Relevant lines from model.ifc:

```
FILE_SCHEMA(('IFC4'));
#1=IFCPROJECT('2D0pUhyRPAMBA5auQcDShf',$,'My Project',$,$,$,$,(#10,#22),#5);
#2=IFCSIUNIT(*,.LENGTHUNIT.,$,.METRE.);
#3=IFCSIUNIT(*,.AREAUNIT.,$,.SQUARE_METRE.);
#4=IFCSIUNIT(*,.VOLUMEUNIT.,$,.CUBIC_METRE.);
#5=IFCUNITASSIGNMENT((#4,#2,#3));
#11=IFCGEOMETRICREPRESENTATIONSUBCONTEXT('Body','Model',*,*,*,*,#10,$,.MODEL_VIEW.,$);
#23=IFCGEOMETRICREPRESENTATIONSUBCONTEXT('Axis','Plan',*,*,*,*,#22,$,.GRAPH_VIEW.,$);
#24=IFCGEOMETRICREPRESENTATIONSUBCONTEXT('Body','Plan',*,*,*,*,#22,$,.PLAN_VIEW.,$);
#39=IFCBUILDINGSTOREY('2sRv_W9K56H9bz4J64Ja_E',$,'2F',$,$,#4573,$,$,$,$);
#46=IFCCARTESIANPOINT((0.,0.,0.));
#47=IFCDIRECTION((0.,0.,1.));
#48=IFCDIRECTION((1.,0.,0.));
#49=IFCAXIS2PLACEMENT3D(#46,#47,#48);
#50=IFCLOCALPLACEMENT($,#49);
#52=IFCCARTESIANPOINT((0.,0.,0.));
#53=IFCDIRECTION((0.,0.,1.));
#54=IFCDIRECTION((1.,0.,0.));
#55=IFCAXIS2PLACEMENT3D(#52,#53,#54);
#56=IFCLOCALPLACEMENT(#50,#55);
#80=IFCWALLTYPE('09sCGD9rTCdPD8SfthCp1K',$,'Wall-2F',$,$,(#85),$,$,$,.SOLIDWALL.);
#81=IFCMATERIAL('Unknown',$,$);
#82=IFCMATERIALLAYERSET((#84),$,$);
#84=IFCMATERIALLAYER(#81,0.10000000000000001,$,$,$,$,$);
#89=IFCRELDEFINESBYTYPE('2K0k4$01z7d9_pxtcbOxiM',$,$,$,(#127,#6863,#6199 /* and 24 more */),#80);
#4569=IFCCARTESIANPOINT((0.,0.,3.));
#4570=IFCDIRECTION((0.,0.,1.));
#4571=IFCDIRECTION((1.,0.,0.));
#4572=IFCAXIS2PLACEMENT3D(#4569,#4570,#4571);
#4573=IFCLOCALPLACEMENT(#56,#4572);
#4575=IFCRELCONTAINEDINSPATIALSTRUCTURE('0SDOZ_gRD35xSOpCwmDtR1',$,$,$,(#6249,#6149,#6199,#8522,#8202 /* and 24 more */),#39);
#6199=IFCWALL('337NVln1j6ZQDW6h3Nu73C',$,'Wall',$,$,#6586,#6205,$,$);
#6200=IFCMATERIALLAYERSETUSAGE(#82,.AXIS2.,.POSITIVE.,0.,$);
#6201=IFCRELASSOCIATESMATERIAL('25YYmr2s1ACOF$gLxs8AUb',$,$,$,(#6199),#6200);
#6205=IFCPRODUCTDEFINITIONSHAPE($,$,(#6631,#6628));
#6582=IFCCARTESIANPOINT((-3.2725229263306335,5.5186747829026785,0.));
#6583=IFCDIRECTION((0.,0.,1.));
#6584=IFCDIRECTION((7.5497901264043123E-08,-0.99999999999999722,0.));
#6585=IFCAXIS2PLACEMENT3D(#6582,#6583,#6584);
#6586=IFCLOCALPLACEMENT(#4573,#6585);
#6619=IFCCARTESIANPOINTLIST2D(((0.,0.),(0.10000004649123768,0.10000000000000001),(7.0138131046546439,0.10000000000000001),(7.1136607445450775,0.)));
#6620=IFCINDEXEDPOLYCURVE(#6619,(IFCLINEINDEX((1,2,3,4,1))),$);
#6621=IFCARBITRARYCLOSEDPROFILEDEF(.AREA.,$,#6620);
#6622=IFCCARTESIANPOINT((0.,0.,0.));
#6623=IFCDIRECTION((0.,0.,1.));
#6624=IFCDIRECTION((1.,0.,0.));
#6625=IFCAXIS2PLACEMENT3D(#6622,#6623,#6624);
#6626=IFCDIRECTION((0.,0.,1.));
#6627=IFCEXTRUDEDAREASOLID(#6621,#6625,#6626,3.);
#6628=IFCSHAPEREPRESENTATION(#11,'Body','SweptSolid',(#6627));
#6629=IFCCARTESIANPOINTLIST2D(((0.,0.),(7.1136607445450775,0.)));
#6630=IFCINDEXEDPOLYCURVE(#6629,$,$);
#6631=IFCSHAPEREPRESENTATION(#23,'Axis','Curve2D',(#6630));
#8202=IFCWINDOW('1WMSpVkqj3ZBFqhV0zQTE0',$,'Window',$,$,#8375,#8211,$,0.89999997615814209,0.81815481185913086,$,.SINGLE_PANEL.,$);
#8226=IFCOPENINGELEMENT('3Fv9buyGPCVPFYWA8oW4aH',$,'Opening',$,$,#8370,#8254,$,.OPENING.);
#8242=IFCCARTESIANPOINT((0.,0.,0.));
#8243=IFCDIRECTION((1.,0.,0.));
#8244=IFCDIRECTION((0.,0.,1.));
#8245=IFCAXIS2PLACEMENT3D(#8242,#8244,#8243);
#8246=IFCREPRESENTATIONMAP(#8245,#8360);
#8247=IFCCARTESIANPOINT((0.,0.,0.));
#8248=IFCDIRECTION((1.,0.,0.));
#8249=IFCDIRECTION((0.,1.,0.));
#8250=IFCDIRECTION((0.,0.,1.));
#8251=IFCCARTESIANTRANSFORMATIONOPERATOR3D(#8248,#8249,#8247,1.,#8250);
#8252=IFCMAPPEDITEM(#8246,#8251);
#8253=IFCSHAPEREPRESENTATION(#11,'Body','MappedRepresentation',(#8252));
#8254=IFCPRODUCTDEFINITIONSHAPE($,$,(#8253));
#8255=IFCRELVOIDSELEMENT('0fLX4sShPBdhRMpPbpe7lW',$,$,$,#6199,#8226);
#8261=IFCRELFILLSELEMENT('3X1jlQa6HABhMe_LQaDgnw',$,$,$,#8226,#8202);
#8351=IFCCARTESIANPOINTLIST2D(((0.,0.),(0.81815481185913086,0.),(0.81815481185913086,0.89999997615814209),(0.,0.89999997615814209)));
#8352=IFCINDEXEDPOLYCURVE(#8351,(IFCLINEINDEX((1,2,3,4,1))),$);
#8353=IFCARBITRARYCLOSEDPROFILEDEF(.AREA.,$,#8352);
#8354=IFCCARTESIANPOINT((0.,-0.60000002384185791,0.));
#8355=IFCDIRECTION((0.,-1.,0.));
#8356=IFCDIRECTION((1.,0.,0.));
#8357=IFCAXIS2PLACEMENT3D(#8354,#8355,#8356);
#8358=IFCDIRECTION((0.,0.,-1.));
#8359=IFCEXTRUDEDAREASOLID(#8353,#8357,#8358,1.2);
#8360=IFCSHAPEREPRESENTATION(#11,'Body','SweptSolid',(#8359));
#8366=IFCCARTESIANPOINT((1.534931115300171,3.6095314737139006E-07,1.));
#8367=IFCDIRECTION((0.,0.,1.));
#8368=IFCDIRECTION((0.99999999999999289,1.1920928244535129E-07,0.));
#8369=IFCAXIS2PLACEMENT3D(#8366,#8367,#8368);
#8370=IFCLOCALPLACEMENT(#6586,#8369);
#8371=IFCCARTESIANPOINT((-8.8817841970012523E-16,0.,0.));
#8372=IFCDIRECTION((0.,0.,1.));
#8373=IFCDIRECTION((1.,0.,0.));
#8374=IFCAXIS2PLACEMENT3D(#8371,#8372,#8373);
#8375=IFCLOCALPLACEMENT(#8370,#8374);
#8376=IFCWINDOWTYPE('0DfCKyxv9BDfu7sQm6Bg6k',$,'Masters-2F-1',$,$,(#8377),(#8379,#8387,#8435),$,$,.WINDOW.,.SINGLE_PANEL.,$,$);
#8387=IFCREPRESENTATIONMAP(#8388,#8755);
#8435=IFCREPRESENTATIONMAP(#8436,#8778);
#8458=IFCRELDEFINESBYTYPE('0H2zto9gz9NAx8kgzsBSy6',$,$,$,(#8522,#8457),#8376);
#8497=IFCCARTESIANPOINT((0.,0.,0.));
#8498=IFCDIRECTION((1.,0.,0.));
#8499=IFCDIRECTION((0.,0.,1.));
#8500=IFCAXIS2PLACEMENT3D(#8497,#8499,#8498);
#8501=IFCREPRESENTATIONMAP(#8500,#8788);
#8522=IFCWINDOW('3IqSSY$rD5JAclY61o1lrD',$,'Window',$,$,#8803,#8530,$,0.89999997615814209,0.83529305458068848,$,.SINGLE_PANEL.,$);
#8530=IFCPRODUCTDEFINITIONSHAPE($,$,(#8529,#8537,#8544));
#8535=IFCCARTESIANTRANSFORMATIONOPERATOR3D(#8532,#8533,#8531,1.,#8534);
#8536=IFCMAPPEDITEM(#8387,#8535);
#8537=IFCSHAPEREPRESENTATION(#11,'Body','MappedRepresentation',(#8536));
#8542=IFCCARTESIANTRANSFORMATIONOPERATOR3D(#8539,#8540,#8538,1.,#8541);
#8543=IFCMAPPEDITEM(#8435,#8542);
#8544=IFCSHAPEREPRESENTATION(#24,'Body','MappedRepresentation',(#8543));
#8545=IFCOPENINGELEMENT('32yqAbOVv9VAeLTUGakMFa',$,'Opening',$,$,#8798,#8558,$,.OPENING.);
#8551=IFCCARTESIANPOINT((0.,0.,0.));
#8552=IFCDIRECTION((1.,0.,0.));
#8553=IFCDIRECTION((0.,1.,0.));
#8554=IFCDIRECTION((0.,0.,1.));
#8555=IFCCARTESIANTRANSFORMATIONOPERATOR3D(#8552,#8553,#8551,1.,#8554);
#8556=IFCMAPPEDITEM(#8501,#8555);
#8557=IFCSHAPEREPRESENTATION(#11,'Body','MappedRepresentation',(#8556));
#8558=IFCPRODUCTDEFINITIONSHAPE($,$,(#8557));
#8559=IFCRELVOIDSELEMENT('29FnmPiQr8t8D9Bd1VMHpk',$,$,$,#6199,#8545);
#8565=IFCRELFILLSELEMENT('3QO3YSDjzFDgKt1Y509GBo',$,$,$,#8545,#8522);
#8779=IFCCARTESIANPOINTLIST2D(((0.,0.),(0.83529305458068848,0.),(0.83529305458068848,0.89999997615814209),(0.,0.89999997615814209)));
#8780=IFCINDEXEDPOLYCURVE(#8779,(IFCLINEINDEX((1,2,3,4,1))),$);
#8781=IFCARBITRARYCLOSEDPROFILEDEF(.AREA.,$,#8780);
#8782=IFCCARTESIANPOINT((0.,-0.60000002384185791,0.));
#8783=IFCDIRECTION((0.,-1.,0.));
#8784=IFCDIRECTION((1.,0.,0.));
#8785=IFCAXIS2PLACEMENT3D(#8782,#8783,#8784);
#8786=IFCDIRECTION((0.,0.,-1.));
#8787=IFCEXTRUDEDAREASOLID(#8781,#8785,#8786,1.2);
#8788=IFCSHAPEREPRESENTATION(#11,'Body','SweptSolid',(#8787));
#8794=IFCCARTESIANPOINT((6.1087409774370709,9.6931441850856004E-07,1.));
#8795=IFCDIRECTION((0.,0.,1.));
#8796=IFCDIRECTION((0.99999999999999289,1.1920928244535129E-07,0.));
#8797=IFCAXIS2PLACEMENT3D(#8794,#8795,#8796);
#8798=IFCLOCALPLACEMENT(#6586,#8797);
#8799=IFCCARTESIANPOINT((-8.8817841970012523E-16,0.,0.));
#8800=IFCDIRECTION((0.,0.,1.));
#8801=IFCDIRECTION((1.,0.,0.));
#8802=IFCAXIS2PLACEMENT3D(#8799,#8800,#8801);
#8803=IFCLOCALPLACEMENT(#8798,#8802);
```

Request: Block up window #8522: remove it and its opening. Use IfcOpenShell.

```python
import ifcopenshell
import ifcopenshell.api.feature
import ifcopenshell.api.root
import ifcopenshell.geom
import ifcopenshell.util.shape

model = ifcopenshell.open("model.ifc")
settings = ifcopenshell.geom.settings()


def volume(element):
    """Net volume in cubic metres, openings subtracted."""
    shape = ifcopenshell.geom.create_shape(settings, element)
    return ifcopenshell.util.shape.get_volume(shape.geometry)


window = model.by_guid("3IqSSY$rD5JAclY61o1lrD")
opening = window.FillsVoids[0].RelatingOpeningElement
wall = opening.VoidsElements[0].RelatingBuildingElement
before = volume(wall)

ifcopenshell.api.root.remove_product(model, product=window)
ifcopenshell.api.feature.remove_feature(model, feature=opening)

after = volume(wall)

print(f"wall volume {before:.3f} -> {after:.3f} m3")

model.write("model-out.ifc")
```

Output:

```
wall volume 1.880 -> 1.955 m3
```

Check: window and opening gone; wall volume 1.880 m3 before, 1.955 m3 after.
